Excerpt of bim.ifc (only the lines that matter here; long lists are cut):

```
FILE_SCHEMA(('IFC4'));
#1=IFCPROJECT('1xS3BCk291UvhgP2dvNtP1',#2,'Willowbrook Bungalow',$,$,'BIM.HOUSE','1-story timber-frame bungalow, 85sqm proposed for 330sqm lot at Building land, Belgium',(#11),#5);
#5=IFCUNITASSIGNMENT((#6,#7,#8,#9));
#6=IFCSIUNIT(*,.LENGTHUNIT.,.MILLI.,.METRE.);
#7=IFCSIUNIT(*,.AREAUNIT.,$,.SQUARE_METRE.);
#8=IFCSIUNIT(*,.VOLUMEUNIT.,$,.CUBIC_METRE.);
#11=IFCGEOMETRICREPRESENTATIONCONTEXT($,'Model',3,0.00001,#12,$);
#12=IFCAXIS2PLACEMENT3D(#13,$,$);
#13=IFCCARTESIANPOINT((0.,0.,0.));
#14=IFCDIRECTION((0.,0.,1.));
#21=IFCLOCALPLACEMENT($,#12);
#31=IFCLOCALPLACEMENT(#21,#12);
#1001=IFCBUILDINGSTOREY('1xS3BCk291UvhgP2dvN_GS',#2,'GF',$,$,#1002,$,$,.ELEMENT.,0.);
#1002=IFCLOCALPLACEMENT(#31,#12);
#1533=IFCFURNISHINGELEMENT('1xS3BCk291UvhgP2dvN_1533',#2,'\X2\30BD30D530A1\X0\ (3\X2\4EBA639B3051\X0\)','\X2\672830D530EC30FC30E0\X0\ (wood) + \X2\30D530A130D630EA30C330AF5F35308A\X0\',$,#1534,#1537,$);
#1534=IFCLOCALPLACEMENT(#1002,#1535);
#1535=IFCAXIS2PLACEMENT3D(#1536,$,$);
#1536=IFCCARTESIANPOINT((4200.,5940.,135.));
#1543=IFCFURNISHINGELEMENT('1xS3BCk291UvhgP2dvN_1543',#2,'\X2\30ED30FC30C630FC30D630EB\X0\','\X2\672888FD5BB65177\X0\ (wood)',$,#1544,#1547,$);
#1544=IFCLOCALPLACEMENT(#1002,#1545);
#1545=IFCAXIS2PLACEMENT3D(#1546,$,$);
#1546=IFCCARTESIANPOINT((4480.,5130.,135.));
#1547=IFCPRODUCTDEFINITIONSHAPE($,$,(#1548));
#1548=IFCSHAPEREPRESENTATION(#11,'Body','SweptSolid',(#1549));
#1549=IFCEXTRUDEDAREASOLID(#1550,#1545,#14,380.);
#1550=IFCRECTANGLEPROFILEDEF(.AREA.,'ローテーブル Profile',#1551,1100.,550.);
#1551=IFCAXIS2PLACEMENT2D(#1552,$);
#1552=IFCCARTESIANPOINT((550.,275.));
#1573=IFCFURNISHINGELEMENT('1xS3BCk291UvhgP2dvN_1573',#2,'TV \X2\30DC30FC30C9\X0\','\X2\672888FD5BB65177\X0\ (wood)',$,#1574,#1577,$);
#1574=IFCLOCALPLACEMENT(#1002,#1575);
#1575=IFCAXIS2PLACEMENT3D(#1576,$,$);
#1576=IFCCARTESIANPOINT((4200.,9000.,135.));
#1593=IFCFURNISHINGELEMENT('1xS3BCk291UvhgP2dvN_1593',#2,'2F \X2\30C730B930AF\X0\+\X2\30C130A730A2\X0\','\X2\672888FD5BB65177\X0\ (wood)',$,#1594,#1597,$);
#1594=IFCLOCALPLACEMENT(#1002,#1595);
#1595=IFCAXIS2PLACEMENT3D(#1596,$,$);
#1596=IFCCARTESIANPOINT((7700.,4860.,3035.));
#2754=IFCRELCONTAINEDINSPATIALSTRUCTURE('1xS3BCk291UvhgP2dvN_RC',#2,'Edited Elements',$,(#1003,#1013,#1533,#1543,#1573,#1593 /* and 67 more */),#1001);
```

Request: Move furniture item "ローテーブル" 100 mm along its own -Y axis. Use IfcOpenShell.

```python
import ifcopenshell
import ifcopenshell.api.geometry
import ifcopenshell.util.placement
import ifcopenshell.util.unit

model = ifcopenshell.open("bim.ifc")
unit_scale = ifcopenshell.util.unit.calculate_unit_scale(model)

item = model.by_guid("1xS3BCk291UvhgP2dvN_1543")
matrix = ifcopenshell.util.placement.get_local_placement(item.ObjectPlacement)
matrix[:3, 3] -= matrix[:3, 1] * 0.1 / unit_scale
ifcopenshell.api.geometry.edit_object_placement(model, product=item, matrix=matrix, is_si=False)

print(ifcopenshell.util.placement.get_local_placement(item.ObjectPlacement).round(3) + 0.0)

model.write("bim-out.ifc")
```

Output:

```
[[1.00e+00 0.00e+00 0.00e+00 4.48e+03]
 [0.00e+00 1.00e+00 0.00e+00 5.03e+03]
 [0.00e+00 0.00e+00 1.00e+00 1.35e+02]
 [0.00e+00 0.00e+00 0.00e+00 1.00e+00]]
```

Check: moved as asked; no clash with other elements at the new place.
